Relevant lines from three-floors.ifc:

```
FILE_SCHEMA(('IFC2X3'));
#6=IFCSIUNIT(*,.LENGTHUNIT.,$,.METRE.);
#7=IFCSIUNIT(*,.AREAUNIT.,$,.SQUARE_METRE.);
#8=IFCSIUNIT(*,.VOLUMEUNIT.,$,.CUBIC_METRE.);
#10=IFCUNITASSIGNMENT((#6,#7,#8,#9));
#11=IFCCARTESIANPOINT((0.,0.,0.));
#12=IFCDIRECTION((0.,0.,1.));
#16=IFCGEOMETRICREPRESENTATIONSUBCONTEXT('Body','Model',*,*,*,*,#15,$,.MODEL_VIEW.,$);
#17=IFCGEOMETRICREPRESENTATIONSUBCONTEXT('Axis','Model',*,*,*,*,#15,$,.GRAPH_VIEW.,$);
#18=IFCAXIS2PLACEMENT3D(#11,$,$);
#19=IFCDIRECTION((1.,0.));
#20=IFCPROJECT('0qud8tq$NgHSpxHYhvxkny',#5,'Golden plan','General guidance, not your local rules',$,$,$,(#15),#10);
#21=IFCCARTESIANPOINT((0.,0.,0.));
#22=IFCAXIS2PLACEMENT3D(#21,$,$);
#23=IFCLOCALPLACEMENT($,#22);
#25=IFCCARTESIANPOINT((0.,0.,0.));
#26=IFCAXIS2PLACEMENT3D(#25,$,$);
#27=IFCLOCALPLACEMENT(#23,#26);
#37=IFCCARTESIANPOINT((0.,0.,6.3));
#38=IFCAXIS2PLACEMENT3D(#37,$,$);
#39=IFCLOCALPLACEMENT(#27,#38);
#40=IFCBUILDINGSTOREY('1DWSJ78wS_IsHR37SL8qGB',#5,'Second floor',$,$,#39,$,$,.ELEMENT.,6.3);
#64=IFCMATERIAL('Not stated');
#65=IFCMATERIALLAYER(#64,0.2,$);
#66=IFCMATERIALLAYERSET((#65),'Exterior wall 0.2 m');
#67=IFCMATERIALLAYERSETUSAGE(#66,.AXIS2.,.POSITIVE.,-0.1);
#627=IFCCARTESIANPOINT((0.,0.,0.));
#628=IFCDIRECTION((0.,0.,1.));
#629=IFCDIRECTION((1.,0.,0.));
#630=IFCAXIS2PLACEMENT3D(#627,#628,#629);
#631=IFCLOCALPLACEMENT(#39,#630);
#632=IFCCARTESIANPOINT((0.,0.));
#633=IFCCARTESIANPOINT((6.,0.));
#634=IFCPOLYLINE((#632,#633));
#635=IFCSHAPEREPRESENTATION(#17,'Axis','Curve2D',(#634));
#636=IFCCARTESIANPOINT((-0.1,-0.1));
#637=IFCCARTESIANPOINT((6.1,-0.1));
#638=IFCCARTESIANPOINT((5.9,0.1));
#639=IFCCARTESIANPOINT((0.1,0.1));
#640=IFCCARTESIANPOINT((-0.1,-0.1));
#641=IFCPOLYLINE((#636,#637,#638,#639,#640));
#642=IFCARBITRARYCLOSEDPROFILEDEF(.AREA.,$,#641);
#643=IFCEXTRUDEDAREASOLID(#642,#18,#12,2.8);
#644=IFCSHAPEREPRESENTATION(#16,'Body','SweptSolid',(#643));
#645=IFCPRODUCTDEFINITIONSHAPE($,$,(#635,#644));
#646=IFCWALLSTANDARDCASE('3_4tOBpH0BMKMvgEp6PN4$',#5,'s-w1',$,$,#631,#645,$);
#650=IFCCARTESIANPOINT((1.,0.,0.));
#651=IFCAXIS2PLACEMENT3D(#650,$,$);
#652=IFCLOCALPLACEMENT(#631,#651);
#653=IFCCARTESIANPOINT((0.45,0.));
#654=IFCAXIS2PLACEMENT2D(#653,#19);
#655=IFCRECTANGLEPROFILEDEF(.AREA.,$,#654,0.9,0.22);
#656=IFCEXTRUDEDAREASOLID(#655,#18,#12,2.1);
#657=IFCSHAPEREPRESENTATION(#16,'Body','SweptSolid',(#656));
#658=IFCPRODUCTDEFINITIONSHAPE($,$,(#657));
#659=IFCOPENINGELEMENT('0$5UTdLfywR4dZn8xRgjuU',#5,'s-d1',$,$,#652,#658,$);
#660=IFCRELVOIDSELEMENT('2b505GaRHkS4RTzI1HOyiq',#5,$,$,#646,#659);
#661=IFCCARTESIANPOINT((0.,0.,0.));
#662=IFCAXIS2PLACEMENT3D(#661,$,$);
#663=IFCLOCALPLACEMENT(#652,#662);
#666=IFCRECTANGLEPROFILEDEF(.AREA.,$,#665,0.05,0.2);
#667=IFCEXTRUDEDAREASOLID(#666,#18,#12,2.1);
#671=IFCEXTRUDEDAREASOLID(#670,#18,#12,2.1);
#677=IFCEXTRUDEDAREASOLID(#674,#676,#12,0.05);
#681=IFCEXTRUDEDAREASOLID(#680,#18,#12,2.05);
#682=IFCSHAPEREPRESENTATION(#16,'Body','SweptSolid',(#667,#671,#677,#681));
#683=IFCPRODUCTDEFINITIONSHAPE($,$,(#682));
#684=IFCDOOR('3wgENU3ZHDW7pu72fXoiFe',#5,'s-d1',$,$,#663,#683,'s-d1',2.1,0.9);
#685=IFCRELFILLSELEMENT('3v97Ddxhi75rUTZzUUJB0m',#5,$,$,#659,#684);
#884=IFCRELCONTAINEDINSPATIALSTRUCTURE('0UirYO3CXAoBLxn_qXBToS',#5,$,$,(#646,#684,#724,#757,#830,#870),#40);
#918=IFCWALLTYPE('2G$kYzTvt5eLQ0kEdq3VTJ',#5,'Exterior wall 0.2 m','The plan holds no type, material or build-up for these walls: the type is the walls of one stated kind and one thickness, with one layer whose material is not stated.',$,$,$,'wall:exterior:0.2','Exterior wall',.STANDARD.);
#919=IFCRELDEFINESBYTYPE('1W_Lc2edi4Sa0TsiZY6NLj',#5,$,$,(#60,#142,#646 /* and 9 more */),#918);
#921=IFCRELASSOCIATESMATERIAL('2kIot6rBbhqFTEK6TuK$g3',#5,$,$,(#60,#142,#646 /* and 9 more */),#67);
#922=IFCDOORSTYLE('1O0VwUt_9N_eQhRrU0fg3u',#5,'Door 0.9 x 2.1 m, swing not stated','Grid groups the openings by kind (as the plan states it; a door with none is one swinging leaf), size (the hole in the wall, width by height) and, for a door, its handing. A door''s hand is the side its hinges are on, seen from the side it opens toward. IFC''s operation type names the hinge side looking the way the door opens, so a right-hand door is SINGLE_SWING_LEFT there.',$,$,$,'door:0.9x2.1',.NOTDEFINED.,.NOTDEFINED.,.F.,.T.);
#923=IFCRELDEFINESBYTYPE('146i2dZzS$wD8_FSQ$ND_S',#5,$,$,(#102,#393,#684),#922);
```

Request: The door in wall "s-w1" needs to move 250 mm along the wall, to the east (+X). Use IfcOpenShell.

```python
import ifcopenshell
import ifcopenshell.api.geometry
import ifcopenshell.util.placement
import ifcopenshell.util.unit

model = ifcopenshell.open("three-floors.ifc")
unit_scale = ifcopenshell.util.unit.calculate_unit_scale(model)

door = model.by_id(684)
opening = door.FillsVoids[0].RelatingOpeningElement
wall = opening.VoidsElements[0].RelatingBuildingElement

wall_matrix = ifcopenshell.util.placement.get_local_placement(wall.ObjectPlacement)
shift = wall_matrix[:3, 0] * 0.25 / unit_scale
before = ifcopenshell.util.placement.get_local_placement(door.ObjectPlacement)[:3, 3].copy()

# The door is placed relative to its opening, so it follows when the opening moves.
matrix = ifcopenshell.util.placement.get_local_placement(opening.ObjectPlacement)
matrix[:3, 3] += shift
ifcopenshell.api.geometry.edit_object_placement(
    model, product=opening, matrix=matrix, is_si=False, should_transform_children=True
)

after = ifcopenshell.util.placement.get_local_placement(door.ObjectPlacement)[:3, 3]
print("door moved by", (after - before).round(3) + 0.0)

model.write("three-floors_edited.ifc")
```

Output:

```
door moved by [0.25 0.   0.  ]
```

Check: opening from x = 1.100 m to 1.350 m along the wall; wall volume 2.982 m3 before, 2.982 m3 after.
